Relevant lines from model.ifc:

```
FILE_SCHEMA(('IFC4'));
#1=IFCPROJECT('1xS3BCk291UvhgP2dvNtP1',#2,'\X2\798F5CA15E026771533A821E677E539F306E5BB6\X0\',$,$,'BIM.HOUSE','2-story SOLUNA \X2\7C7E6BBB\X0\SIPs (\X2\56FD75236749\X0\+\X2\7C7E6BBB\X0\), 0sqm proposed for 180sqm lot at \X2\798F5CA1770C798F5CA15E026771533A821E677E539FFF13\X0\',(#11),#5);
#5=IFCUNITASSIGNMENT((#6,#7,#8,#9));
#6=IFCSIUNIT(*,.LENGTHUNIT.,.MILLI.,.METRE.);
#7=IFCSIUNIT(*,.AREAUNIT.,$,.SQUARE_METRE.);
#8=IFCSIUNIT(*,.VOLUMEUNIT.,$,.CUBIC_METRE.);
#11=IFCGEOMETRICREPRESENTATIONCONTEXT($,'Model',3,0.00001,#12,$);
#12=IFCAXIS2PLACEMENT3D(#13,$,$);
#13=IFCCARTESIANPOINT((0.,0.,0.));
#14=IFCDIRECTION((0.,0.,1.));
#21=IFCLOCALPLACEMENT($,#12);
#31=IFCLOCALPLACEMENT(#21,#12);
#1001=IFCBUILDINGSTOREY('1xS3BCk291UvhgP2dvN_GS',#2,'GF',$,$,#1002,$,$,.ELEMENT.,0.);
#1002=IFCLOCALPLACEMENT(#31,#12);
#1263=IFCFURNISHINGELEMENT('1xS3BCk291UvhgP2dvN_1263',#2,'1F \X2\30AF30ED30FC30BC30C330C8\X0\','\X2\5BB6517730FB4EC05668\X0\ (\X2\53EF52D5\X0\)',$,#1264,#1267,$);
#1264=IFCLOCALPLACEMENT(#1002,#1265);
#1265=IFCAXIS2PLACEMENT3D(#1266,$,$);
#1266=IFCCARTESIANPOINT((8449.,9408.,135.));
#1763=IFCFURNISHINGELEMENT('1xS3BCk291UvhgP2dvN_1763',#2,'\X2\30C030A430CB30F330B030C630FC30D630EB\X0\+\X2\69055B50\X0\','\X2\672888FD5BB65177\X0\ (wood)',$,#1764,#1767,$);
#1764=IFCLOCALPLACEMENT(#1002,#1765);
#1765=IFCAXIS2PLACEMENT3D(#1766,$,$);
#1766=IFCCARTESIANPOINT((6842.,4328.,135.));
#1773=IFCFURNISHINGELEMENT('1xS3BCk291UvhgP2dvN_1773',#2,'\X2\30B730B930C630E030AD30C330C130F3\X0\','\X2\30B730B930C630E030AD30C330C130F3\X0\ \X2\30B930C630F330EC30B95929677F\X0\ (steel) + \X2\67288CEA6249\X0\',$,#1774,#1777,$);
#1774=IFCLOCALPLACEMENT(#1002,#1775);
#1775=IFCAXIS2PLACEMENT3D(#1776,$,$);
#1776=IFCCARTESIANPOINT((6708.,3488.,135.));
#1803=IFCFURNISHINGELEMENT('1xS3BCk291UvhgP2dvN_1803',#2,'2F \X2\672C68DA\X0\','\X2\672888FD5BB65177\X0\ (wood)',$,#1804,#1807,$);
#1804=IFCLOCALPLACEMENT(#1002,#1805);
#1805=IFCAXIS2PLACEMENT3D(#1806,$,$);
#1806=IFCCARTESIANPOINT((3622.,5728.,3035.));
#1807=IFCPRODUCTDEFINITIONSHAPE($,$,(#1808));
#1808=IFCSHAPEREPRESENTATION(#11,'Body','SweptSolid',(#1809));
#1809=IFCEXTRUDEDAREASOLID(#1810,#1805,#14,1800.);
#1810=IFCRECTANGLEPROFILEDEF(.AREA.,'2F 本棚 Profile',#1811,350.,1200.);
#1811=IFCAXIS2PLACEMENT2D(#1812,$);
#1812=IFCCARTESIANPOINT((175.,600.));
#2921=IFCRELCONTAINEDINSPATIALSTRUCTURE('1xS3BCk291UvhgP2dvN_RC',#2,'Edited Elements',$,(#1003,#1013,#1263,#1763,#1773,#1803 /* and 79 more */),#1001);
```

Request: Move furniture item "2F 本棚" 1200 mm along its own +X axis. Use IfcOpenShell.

```python
import ifcopenshell
import ifcopenshell.api.geometry
import ifcopenshell.util.placement
import ifcopenshell.util.unit

model = ifcopenshell.open("model.ifc")
unit_scale = ifcopenshell.util.unit.calculate_unit_scale(model)

item = model.by_id(1803)
matrix = ifcopenshell.util.placement.get_local_placement(item.ObjectPlacement)
matrix[:3, 3] += matrix[:3, 0] * 1.2 / unit_scale
ifcopenshell.api.geometry.edit_object_placement(model, product=item, matrix=matrix, is_si=False)

print(ifcopenshell.util.placement.get_local_placement(item.ObjectPlacement).round(3) + 0.0)

model.write("model-out.ifc")
```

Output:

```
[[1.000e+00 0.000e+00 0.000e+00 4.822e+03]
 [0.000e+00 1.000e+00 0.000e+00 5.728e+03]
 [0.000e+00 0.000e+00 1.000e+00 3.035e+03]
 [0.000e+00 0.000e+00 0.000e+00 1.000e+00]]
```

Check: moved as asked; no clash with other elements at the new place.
